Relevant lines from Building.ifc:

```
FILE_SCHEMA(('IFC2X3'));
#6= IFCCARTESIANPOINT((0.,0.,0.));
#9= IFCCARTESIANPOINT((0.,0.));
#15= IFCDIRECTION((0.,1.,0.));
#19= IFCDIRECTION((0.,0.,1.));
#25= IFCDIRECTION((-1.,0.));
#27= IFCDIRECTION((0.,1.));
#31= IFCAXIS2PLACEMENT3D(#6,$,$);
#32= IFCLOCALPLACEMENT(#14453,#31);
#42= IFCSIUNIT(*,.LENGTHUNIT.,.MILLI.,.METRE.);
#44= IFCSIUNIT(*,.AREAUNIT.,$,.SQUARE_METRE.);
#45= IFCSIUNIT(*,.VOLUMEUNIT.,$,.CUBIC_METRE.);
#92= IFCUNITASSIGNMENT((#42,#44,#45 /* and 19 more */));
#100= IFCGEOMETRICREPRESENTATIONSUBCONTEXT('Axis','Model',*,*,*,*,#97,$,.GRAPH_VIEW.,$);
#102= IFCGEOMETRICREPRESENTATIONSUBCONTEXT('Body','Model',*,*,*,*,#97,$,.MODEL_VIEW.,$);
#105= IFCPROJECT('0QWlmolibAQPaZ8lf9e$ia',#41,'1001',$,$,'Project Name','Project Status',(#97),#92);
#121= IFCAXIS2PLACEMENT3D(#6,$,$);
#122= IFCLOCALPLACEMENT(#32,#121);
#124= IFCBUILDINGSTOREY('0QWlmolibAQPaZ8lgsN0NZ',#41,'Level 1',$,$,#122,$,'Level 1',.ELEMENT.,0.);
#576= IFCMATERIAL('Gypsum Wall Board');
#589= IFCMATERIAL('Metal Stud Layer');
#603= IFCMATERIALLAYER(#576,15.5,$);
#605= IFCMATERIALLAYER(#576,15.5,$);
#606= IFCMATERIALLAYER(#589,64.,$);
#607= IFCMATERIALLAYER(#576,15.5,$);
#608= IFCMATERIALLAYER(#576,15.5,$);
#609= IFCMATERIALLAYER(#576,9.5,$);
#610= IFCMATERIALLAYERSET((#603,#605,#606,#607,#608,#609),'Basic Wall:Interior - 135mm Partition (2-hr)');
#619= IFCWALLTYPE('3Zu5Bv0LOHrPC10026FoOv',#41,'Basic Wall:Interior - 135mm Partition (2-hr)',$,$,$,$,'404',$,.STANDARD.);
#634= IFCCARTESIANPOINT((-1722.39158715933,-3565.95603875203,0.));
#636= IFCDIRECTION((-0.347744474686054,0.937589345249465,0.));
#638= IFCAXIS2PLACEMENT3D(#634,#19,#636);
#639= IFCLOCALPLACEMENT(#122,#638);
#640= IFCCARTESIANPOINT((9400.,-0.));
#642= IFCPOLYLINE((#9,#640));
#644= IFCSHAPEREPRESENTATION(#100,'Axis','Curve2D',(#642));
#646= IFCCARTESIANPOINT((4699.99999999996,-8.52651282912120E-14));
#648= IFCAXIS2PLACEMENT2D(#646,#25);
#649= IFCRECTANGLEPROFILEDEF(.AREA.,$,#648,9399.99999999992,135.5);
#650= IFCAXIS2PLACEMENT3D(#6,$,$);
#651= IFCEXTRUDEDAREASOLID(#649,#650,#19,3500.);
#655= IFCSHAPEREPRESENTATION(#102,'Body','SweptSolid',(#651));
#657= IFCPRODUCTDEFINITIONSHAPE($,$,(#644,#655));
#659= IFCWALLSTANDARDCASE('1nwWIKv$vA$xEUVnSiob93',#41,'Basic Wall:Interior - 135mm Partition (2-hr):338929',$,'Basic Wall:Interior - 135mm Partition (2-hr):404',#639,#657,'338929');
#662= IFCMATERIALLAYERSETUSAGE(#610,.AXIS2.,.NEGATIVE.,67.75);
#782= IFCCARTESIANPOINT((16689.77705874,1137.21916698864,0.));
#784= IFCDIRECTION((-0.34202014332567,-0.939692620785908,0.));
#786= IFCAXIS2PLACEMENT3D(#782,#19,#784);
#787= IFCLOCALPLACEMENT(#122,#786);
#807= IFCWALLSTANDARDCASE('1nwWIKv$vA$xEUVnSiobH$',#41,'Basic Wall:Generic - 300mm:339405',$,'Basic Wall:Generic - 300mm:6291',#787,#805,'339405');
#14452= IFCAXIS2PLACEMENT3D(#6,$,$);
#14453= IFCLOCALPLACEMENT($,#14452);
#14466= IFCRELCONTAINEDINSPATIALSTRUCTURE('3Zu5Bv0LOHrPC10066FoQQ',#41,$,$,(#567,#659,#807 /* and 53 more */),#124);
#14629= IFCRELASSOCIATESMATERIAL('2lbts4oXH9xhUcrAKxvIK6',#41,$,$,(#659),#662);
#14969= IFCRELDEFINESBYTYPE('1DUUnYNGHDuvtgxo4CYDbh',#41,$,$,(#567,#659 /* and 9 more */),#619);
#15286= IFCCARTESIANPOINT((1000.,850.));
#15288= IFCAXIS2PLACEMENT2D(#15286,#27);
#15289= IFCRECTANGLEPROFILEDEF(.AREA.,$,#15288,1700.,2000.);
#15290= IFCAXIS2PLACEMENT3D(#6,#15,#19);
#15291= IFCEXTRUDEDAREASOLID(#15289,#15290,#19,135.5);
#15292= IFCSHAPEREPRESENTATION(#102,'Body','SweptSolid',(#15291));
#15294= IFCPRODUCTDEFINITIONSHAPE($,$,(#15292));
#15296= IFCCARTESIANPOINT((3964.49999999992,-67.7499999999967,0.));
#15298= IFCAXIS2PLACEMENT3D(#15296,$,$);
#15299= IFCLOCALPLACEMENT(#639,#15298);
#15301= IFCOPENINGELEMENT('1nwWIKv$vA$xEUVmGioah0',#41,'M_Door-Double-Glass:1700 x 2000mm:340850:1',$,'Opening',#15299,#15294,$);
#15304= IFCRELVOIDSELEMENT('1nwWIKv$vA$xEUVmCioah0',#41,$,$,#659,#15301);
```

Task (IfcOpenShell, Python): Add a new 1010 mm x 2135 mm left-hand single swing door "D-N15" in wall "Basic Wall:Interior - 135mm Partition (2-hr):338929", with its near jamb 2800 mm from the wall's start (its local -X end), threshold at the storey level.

```python
import numpy as np
import ifcopenshell
import ifcopenshell.api.feature
import ifcopenshell.api.geometry
import ifcopenshell.api.root
import ifcopenshell.api.spatial
import ifcopenshell.api.type
import ifcopenshell.geom
import ifcopenshell.util.element
import ifcopenshell.util.placement
import ifcopenshell.util.representation
import ifcopenshell.util.shape
import ifcopenshell.util.unit

model = ifcopenshell.open("Building.ifc")
unit_scale = ifcopenshell.util.unit.calculate_unit_scale(model)
settings = ifcopenshell.geom.settings()


def volume(element):
    """Net volume in cubic metres, openings subtracted."""
    shape = ifcopenshell.geom.create_shape(settings, element)
    return ifcopenshell.util.shape.get_volume(shape.geometry)


wall = model.by_guid("1nwWIKv$vA$xEUVnSiob93")
storey = ifcopenshell.util.element.get_container(wall, ifc_class="IfcBuildingStorey")
context = ifcopenshell.util.representation.get_context(model, "Model", "Body", "MODEL_VIEW")
before = volume(wall)

width, height, from_end, sill = 1.01, 2.135, 2.8, 0.0  # metres

# The wall runs along its own X axis, and the end named is its -X end.
wall_shape = ifcopenshell.geom.create_shape(settings, wall)
x, y, z = ifcopenshell.util.shape.get_vertices(wall_shape.geometry).T
start = x.min() + from_end
face, thickness = float(y.min()), float(y.max() - y.min())
wall_matrix = ifcopenshell.util.placement.get_local_placement(wall.ObjectPlacement)
level = ifcopenshell.util.placement.get_local_placement(storey.ObjectPlacement)[2, 3]


def in_wall(x, y):
    """Placement at x, y metres in the wall's axes, at sill height."""
    matrix = wall_matrix.copy()
    matrix[:, 3] = wall_matrix @ np.array([x / unit_scale, y / unit_scale, 0.0, 1.0])
    matrix[2, 3] = level + sill / unit_scale
    return matrix


# Opening: a box that overshoots both wall faces by 50 mm.
opening = ifcopenshell.api.root.create_entity(model, ifc_class="IfcOpeningElement")
box = ifcopenshell.api.geometry.add_wall_representation(
    model, context=context, length=width, height=height, thickness=thickness + 0.1
)
ifcopenshell.api.geometry.assign_representation(model, product=opening, representation=box)
ifcopenshell.api.geometry.edit_object_placement(model, product=opening, matrix=in_wall(start, face - 0.05), is_si=False)
ifcopenshell.api.feature.add_feature(model, feature=opening, element=wall)

door = ifcopenshell.api.root.create_entity(model, ifc_class="IfcDoor", name="D-N15")
door.OverallWidth, door.OverallHeight = width / unit_scale, height / unit_scale
body = ifcopenshell.api.geometry.add_door_representation(
    model,
    context=context,
    overall_width=door.OverallWidth,
    overall_height=door.OverallHeight,
    operation_type="SINGLE_SWING_LEFT",
    lining_properties={"LiningDepth": thickness / unit_scale, "ThresholdDepth": thickness / unit_scale},
)
ifcopenshell.api.geometry.assign_representation(model, product=door, representation=body)
ifcopenshell.api.spatial.assign_container(model, products=[door], relating_structure=storey)
fills = ifcopenshell.api.feature.add_filling(model, opening=opening, element=door)
fills.OwnerHistory = door.OwnerHistory  # required in IFC2X3

# IFC2X3 keeps the operation on the door style.
style = ifcopenshell.api.root.create_entity(model, ifc_class="IfcDoorStyle", name="D-N15")
style.OperationType, style.ConstructionType = "SINGLE_SWING_LEFT", "NOTDEFINED"
style.ParameterTakesPrecedence = style.Sizeable = False
ifcopenshell.api.type.assign_type(model, related_objects=[door], relating_type=style)

# The lining spans the wall, so the door starts at the wall face.
ifcopenshell.api.geometry.edit_object_placement(model, product=door, matrix=in_wall(start, face), is_si=False)

after = volume(wall)

print(f"wall volume {before:.3f} -> {after:.3f} m3")

model.write("Building_edited.ifc")
```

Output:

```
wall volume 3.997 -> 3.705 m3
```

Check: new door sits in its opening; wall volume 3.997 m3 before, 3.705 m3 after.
